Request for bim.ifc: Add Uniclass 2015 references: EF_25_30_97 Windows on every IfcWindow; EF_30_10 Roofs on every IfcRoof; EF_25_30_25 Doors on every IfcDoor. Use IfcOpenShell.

First a look at what the model holds.

```python
import ifcopenshell

model = ifcopenshell.open("bim.ifc")
print(model.schema)
print("classifications:", [c.Name for c in model.by_type("IfcClassification")])
for ifc_class in ("IfcDoor", "IfcRoof", "IfcStair", "IfcWall", "IfcWindow"):
    print(ifc_class, len(model.by_type(ifc_class)))
```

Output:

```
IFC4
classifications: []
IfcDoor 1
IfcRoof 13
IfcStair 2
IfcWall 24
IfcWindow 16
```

```python
import ifcopenshell
import ifcopenshell.api.classification

model = ifcopenshell.open("bim.ifc")

system = ifcopenshell.api.classification.add_classification(model, classification="Uniclass 2015")

codes = {
    "IfcWindow": ("EF_25_30_97", "Windows"),
    "IfcRoof": ("EF_30_10", "Roofs"),
    "IfcDoor": ("EF_25_30_25", "Doors"),
}
for ifc_class, (code, name) in codes.items():
    products = model.by_type(ifc_class)
    ifcopenshell.api.classification.add_reference(
        model, products=products, classification=system, identification=code, name=name
    )
    print(code, len(products))

model.write("bim_v2.ifc")
```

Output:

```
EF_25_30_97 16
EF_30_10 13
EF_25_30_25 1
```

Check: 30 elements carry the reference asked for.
